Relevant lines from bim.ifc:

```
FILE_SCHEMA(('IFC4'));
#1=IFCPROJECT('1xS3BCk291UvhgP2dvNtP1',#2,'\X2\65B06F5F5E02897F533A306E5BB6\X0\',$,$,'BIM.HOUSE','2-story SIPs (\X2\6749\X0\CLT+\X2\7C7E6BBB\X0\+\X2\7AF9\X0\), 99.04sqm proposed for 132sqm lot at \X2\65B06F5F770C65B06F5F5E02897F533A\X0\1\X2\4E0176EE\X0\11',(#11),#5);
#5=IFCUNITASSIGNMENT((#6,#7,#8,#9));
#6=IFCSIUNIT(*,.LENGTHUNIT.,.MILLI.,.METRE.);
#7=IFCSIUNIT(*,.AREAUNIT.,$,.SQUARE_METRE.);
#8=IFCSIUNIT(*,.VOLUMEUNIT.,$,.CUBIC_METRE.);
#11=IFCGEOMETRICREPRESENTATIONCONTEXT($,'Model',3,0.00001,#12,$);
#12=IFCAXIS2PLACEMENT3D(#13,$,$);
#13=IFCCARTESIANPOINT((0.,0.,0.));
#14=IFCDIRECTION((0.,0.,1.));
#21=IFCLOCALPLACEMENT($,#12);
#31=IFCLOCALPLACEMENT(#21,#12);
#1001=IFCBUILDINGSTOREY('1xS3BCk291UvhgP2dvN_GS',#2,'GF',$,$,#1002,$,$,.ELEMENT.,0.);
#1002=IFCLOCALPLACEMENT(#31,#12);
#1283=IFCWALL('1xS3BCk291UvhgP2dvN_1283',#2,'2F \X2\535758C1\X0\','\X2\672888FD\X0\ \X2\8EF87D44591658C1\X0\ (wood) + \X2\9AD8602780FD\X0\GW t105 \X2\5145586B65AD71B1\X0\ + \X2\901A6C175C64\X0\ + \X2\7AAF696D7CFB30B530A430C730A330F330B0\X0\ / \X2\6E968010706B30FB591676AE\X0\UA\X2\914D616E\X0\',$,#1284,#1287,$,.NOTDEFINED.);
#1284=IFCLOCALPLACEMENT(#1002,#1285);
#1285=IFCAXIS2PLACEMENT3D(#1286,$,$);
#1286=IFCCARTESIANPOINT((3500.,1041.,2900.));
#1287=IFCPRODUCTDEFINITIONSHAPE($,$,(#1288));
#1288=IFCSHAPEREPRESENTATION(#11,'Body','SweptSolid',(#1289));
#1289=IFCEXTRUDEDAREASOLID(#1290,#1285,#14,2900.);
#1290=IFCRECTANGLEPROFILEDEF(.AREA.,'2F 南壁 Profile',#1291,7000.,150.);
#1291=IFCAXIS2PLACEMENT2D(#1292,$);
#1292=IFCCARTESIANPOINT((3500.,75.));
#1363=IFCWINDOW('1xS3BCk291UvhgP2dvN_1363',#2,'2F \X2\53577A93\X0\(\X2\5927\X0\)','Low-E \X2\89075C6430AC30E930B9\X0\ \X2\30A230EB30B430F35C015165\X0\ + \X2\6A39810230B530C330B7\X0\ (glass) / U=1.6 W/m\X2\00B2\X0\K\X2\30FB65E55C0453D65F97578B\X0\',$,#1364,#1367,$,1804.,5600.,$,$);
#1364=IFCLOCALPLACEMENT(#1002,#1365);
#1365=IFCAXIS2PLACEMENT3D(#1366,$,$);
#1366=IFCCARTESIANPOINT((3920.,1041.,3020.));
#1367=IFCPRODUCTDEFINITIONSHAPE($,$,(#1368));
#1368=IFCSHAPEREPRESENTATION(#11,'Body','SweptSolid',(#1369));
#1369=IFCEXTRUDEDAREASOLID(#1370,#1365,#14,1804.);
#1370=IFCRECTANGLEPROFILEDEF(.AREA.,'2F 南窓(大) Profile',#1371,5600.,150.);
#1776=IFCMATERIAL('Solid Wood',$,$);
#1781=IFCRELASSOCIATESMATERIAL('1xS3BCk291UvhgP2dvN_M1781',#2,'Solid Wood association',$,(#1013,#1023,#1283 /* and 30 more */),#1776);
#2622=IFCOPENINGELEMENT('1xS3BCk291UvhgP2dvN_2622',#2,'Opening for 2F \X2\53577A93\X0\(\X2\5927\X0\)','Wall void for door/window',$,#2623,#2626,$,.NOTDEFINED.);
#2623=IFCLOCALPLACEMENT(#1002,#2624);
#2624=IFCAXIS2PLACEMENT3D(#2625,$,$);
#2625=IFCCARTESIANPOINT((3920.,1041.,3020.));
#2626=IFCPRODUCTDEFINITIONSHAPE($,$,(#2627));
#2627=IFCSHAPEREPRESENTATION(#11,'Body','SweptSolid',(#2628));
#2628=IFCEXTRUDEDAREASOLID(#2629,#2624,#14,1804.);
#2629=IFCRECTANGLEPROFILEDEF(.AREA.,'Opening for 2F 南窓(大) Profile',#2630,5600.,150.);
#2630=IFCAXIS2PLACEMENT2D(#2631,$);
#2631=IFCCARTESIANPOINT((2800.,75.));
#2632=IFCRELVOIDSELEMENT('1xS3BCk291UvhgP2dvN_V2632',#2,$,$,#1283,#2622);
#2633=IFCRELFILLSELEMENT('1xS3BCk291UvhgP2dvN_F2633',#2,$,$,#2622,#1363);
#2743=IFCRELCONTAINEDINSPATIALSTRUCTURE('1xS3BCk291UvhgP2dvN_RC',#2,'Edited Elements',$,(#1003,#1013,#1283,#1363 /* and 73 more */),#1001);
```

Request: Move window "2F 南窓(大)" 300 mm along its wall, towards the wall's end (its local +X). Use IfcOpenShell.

```python
import ifcopenshell
import ifcopenshell.api.geometry
import ifcopenshell.util.placement

model = ifcopenshell.open("bim.ifc")

window = model.by_guid("1xS3BCk291UvhgP2dvN_1363")
opening = window.FillsVoids[0].RelatingOpeningElement
wall = opening.VoidsElements[0].RelatingBuildingElement

wall_matrix = ifcopenshell.util.placement.get_local_placement(wall.ObjectPlacement)
shift = wall_matrix[:3, 0] * 300.0
before = ifcopenshell.util.placement.get_local_placement(window.ObjectPlacement)[:3, 3].copy()

# The window is not placed relative to its opening, so move both.
for product in (opening, window):
    matrix = ifcopenshell.util.placement.get_local_placement(product.ObjectPlacement)
    matrix[:3, 3] += shift
    ifcopenshell.api.geometry.edit_object_placement(model, product=product, matrix=matrix, is_si=False)

after = ifcopenshell.util.placement.get_local_placement(window.ObjectPlacement)[:3, 3]
print("window moved by", (after - before).round(3) + 0.0)

model.write("bim_v2.ifc")
```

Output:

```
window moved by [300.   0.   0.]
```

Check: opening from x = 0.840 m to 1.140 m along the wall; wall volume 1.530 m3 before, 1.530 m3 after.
